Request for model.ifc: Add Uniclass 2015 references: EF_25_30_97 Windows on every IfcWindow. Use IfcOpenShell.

First a look at what the model holds.

```python
import ifcopenshell

model = ifcopenshell.open("model.ifc")
print(model.schema)
print("classifications:", [c.Name for c in model.by_type("IfcClassification")])
for ifc_class in ("IfcDoor", "IfcRoof", "IfcStair", "IfcWall", "IfcWindow"):
    print(ifc_class, len(model.by_type(ifc_class)))
```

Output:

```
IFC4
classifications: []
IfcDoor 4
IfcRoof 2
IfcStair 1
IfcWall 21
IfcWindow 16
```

```python
import ifcopenshell
import ifcopenshell.api.classification

model = ifcopenshell.open("model.ifc")

system = ifcopenshell.api.classification.add_classification(model, classification="Uniclass 2015")

codes = {
    "IfcWindow": ("EF_25_30_97", "Windows"),
}
for ifc_class, (code, name) in codes.items():
    products = model.by_type(ifc_class)
    ifcopenshell.api.classification.add_reference(
        model, products=products, classification=system, identification=code, name=name
    )
    print(code, len(products))

model.write("model_v2.ifc")
```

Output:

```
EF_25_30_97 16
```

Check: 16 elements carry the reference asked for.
